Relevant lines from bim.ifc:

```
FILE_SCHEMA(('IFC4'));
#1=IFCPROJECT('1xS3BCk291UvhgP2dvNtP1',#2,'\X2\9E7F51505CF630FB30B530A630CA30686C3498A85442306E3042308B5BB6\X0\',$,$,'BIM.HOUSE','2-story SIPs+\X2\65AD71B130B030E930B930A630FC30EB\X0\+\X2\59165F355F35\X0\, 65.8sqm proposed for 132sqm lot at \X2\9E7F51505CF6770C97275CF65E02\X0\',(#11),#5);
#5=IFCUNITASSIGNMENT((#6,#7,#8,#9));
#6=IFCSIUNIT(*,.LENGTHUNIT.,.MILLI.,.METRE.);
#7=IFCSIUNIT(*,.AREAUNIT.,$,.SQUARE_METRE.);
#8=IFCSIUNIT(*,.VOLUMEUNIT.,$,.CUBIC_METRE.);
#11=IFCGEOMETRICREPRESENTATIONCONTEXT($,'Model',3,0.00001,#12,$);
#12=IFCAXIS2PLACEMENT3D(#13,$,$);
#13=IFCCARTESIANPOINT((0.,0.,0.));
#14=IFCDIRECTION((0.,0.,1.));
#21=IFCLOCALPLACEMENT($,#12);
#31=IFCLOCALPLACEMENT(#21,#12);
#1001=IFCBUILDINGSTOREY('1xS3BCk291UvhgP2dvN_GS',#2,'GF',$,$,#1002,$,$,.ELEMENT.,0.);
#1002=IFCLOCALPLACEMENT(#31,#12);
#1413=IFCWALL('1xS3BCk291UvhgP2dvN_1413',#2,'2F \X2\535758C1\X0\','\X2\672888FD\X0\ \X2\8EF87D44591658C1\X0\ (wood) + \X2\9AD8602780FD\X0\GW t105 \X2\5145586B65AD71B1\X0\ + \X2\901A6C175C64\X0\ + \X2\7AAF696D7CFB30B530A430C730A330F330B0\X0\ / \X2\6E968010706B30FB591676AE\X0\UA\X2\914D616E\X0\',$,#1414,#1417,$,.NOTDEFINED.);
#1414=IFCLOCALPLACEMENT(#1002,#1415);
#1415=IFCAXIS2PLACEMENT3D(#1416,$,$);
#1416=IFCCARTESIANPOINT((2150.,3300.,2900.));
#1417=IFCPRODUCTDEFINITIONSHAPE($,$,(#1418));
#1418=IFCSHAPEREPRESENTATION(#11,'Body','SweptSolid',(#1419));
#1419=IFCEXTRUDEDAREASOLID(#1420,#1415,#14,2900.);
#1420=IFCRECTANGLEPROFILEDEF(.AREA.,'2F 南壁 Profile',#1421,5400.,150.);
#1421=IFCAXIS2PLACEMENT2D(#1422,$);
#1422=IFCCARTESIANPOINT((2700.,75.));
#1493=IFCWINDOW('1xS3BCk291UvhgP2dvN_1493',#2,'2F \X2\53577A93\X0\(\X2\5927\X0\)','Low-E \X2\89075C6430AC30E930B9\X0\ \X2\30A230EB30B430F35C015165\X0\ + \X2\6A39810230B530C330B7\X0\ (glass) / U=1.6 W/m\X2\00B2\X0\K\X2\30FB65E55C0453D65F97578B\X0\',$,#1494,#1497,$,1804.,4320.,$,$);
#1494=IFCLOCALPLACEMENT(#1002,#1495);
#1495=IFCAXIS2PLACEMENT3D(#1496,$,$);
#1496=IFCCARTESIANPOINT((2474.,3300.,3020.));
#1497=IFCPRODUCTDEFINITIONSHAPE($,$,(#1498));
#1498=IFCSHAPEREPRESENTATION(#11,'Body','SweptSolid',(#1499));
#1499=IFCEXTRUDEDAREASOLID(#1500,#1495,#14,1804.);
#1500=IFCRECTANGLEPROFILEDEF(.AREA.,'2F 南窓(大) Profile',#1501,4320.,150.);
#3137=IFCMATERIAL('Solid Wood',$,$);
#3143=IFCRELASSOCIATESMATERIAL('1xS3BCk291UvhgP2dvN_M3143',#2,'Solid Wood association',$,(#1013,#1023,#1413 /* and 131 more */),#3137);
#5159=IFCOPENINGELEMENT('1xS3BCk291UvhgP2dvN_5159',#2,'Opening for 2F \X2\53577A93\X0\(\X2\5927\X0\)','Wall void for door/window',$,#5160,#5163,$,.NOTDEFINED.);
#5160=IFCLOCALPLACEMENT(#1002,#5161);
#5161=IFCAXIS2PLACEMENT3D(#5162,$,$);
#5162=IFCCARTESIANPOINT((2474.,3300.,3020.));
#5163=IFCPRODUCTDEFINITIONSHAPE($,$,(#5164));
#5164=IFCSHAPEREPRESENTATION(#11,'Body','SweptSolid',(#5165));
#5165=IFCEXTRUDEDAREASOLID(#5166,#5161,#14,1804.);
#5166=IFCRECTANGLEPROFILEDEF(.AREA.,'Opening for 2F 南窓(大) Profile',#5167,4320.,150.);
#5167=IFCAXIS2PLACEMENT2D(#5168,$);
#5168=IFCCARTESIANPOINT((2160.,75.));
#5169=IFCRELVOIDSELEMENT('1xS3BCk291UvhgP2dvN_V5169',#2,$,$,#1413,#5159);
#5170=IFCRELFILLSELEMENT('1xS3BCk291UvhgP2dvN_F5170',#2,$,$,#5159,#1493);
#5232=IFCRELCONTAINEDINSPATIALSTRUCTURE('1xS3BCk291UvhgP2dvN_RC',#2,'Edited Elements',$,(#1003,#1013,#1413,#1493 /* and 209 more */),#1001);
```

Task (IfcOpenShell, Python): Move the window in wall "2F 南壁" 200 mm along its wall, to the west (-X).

```python
import ifcopenshell
import ifcopenshell.api.geometry
import ifcopenshell.util.placement
import ifcopenshell.util.unit

model = ifcopenshell.open("bim.ifc")
unit_scale = ifcopenshell.util.unit.calculate_unit_scale(model)

window = model.by_id(1493)
opening = window.FillsVoids[0].RelatingOpeningElement
wall = opening.VoidsElements[0].RelatingBuildingElement

wall_matrix = ifcopenshell.util.placement.get_local_placement(wall.ObjectPlacement)
shift = wall_matrix[:3, 0] * -0.2 / unit_scale
before = ifcopenshell.util.placement.get_local_placement(window.ObjectPlacement)[:3, 3].copy()

# The window is not placed relative to its opening, so move both.
for product in (opening, window):
    matrix = ifcopenshell.util.placement.get_local_placement(product.ObjectPlacement)
    matrix[:3, 3] += shift
    ifcopenshell.api.geometry.edit_object_placement(model, product=product, matrix=matrix, is_si=False)

after = ifcopenshell.util.placement.get_local_placement(window.ObjectPlacement)[:3, 3]
print("window moved by", (after - before).round(3) + 0.0)

model.write("bim_v2.ifc")
```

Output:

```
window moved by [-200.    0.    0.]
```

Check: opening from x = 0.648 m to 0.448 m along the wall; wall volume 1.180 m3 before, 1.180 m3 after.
